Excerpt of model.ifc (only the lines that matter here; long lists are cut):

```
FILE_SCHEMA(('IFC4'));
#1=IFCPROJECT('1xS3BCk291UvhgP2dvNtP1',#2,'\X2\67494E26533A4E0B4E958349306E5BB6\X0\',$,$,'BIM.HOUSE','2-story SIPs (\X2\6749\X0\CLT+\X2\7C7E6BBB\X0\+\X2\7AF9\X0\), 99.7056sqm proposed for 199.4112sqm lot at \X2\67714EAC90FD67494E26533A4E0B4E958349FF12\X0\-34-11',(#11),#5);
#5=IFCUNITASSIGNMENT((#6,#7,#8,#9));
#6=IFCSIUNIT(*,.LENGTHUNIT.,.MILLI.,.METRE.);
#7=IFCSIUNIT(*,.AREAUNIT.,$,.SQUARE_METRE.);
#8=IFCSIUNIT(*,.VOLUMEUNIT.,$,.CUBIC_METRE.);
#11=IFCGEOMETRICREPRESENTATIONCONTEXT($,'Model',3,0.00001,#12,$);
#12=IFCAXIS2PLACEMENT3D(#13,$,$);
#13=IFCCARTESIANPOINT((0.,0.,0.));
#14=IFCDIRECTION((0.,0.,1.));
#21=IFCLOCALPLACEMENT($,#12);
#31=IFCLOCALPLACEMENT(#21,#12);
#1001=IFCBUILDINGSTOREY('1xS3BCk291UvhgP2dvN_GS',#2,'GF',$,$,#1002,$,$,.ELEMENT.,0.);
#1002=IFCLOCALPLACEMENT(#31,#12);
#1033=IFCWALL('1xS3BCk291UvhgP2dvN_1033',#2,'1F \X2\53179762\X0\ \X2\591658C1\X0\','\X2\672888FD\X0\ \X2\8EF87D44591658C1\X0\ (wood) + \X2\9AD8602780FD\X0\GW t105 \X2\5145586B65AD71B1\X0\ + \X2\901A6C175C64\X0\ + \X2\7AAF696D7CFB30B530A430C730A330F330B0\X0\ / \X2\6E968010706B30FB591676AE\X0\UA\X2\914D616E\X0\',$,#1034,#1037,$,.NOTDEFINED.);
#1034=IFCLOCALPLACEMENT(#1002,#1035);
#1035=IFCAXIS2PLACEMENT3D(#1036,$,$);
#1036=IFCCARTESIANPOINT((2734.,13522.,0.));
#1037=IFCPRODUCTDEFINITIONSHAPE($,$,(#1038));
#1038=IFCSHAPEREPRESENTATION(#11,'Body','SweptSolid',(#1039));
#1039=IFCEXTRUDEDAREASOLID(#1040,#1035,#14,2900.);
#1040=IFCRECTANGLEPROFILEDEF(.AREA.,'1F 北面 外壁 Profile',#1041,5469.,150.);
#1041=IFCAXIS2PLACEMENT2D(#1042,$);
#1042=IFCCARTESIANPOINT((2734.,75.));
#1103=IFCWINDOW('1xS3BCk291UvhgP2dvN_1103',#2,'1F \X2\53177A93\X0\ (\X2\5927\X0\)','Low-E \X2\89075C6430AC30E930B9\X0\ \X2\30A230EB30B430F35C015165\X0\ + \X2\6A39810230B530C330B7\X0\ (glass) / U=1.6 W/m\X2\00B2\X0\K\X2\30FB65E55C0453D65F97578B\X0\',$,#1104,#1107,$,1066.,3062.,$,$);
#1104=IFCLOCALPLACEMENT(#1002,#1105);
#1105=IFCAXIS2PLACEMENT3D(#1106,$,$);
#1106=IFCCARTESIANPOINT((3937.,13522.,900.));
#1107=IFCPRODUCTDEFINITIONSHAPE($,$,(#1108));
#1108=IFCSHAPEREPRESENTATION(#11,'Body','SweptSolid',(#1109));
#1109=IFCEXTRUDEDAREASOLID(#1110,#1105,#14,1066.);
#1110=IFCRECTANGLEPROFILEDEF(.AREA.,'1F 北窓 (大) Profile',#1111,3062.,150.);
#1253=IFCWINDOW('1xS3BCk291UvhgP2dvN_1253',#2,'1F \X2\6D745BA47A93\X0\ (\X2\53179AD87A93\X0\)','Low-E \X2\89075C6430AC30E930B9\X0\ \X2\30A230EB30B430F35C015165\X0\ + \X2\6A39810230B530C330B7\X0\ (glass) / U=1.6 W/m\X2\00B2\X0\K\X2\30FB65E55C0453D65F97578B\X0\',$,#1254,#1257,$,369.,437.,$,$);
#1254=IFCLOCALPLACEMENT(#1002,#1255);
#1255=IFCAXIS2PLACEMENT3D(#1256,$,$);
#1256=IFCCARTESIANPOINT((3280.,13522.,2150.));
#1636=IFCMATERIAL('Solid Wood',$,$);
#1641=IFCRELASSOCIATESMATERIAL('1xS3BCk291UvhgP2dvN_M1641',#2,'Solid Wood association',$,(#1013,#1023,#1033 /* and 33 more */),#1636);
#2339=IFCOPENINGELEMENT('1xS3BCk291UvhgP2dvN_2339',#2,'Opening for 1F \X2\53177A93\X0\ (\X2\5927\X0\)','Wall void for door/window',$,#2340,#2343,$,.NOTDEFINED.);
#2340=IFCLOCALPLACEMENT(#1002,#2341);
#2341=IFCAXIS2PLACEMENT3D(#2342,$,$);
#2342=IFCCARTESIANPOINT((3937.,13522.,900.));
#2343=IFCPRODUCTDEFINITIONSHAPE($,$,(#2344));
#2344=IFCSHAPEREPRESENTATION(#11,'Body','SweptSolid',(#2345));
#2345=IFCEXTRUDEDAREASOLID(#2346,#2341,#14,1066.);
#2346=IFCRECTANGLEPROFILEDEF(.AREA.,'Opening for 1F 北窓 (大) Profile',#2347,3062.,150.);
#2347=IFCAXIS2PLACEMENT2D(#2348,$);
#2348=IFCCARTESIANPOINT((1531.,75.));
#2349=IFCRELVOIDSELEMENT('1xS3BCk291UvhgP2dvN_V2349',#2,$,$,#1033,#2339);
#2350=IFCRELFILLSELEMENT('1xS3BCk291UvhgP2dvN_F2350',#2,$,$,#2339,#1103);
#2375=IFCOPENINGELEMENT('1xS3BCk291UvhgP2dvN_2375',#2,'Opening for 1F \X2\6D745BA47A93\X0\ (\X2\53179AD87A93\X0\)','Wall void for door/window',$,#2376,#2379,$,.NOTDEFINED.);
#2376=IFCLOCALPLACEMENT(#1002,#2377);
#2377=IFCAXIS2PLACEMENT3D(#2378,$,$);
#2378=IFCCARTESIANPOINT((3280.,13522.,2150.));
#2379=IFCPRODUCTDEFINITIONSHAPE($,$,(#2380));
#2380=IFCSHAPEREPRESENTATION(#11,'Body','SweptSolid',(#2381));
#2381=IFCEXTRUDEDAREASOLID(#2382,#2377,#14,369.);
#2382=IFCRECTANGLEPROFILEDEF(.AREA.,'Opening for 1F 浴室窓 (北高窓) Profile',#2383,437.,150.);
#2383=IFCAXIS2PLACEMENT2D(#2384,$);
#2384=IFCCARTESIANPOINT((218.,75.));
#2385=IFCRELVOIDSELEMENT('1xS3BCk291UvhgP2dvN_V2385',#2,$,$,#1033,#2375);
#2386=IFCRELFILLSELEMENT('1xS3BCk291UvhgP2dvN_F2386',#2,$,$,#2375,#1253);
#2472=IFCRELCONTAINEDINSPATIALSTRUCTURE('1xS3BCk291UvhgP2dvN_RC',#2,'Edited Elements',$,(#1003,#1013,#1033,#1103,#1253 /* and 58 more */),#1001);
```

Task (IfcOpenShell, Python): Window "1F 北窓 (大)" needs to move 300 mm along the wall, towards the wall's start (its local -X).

```python
import ifcopenshell
import ifcopenshell.api.geometry
import ifcopenshell.util.placement

model = ifcopenshell.open("model.ifc")

window = model.by_guid("1xS3BCk291UvhgP2dvN_1103")
opening = window.FillsVoids[0].RelatingOpeningElement
wall = opening.VoidsElements[0].RelatingBuildingElement

wall_matrix = ifcopenshell.util.placement.get_local_placement(wall.ObjectPlacement)
shift = wall_matrix[:3, 0] * -300.0
before = ifcopenshell.util.placement.get_local_placement(window.ObjectPlacement)[:3, 3].copy()

# The window is not placed relative to its opening, so move both.
for product in (opening, window):
    matrix = ifcopenshell.util.placement.get_local_placement(product.ObjectPlacement)
    matrix[:3, 3] += shift
    ifcopenshell.api.geometry.edit_object_placement(model, product=product, matrix=matrix, is_si=False)

after = ifcopenshell.util.placement.get_local_placement(window.ObjectPlacement)[:3, 3]
print("window moved by", (after - before).round(3) + 0.0)

model.write("model_edited.ifc")
```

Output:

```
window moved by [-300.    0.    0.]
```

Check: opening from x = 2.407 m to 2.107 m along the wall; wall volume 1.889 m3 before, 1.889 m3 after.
